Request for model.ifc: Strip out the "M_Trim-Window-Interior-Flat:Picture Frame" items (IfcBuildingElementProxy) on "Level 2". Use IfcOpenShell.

First a look at what the model holds.

```python
import ifcopenshell
import ifcopenshell.util.element

model = ifcopenshell.open("model.ifc")
print(model.schema)
storey = next(s for s in model.by_type("IfcBuildingStorey") if s.Name == "Level 2")
proxies = [e for e in ifcopenshell.util.element.get_decomposition(storey) if e.is_a("IfcBuildingElementProxy")]
seen = {}
for e in proxies:
    element_type = ifcopenshell.util.element.get_type(e)
    name = element_type.Name if element_type not in (None, e) else None
    seen[name] = seen.get(name, 0) + 1
for name, count in sorted(seen.items(), key=str):
    print(count, "x", name)
```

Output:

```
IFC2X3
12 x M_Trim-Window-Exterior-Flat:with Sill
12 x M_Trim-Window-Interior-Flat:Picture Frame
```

```python
import ifcopenshell
import ifcopenshell.api.root
import ifcopenshell.util.element

model = ifcopenshell.open("model.ifc")

storey = next(s for s in model.by_type("IfcBuildingStorey") if s.Name == "Level 2")
proxies = [e for e in ifcopenshell.util.element.get_decomposition(storey) if e.is_a("IfcBuildingElementProxy")]
targets = [e for e in proxies if (t := ifcopenshell.util.element.get_type(e)) not in (None, e) and t.Name == "M_Trim-Window-Interior-Flat:Picture Frame"]

for e in targets:
    ifcopenshell.api.root.remove_product(model, product=e)
print(len(targets), "removed")

model.write("model_updated.ifc")
```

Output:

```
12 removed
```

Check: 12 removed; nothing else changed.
